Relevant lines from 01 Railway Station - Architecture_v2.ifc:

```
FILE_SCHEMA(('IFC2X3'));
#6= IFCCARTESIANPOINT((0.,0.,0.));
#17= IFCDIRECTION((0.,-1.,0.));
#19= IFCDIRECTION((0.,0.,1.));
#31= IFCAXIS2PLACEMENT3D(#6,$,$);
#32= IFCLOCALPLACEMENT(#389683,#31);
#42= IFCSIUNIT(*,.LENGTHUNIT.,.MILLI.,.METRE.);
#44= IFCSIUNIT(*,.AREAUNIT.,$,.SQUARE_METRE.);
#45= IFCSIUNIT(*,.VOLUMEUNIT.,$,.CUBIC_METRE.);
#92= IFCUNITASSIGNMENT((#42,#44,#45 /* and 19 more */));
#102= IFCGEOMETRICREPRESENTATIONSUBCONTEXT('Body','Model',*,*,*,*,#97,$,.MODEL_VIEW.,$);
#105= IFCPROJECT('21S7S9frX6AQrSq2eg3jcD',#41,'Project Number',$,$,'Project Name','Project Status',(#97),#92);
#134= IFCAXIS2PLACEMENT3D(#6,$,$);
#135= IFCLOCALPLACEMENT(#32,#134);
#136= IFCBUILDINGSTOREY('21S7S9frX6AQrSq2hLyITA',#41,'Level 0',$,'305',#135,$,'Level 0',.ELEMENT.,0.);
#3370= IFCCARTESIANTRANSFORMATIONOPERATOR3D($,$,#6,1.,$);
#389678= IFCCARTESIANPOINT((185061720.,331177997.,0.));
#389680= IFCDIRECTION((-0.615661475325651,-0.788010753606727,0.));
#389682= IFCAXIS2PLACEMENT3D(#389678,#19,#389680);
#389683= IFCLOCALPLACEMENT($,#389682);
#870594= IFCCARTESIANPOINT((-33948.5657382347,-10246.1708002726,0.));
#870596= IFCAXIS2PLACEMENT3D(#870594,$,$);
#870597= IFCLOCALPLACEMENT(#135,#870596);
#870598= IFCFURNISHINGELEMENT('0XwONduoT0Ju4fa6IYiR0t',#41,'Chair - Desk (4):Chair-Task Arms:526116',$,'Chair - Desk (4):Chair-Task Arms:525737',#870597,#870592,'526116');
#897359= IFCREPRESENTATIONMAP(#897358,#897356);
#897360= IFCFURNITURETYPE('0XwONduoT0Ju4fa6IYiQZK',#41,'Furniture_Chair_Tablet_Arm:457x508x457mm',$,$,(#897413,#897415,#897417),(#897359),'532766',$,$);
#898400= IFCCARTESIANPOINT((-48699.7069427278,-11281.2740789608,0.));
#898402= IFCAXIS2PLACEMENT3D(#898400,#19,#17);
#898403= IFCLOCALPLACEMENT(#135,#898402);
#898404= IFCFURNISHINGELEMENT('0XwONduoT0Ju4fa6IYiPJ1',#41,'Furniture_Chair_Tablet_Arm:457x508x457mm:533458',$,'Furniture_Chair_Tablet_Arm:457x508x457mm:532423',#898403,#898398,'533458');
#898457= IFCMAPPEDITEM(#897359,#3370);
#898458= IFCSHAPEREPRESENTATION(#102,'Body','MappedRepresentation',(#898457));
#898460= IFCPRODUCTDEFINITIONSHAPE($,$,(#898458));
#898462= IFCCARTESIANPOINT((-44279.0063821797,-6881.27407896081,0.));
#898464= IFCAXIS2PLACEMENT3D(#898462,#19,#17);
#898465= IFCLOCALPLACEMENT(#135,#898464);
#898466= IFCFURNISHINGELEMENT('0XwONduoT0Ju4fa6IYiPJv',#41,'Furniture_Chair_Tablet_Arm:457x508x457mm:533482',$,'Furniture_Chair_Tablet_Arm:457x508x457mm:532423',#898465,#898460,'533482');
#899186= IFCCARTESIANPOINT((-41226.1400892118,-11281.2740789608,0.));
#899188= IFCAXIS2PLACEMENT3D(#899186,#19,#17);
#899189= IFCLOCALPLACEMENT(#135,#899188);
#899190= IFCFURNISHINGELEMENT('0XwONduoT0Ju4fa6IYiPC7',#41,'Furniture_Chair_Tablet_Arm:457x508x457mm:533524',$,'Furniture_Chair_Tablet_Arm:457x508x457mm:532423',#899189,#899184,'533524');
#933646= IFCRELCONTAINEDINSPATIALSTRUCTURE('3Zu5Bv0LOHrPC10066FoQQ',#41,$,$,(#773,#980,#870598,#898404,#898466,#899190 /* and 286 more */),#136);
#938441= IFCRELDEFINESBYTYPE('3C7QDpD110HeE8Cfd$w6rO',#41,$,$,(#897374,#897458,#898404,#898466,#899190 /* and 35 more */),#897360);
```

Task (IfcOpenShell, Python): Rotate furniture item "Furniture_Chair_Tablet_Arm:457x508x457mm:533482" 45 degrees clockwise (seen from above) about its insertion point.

```python
import ifcopenshell
import ifcopenshell.api.geometry
import ifcopenshell.util.placement

model = ifcopenshell.open("01 Railway Station - Architecture_v2.ifc")

item = model.by_guid("0XwONduoT0Ju4fa6IYiPJv")
matrix = ifcopenshell.util.placement.get_local_placement(item.ObjectPlacement)
matrix = matrix @ ifcopenshell.util.placement.rotation(-45, "Z")
ifcopenshell.api.geometry.edit_object_placement(model, product=item, matrix=matrix, is_si=False)

print(ifcopenshell.util.placement.get_local_placement(item.ObjectPlacement).round(3) + 0.0)

model.write("01 Railway Station - Architecture_v2_updated.ifc")
```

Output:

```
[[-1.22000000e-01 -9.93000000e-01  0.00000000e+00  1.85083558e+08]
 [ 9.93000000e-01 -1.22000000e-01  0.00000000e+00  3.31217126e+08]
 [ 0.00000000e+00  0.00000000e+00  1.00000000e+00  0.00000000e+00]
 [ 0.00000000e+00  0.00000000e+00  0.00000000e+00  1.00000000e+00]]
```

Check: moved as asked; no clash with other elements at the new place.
